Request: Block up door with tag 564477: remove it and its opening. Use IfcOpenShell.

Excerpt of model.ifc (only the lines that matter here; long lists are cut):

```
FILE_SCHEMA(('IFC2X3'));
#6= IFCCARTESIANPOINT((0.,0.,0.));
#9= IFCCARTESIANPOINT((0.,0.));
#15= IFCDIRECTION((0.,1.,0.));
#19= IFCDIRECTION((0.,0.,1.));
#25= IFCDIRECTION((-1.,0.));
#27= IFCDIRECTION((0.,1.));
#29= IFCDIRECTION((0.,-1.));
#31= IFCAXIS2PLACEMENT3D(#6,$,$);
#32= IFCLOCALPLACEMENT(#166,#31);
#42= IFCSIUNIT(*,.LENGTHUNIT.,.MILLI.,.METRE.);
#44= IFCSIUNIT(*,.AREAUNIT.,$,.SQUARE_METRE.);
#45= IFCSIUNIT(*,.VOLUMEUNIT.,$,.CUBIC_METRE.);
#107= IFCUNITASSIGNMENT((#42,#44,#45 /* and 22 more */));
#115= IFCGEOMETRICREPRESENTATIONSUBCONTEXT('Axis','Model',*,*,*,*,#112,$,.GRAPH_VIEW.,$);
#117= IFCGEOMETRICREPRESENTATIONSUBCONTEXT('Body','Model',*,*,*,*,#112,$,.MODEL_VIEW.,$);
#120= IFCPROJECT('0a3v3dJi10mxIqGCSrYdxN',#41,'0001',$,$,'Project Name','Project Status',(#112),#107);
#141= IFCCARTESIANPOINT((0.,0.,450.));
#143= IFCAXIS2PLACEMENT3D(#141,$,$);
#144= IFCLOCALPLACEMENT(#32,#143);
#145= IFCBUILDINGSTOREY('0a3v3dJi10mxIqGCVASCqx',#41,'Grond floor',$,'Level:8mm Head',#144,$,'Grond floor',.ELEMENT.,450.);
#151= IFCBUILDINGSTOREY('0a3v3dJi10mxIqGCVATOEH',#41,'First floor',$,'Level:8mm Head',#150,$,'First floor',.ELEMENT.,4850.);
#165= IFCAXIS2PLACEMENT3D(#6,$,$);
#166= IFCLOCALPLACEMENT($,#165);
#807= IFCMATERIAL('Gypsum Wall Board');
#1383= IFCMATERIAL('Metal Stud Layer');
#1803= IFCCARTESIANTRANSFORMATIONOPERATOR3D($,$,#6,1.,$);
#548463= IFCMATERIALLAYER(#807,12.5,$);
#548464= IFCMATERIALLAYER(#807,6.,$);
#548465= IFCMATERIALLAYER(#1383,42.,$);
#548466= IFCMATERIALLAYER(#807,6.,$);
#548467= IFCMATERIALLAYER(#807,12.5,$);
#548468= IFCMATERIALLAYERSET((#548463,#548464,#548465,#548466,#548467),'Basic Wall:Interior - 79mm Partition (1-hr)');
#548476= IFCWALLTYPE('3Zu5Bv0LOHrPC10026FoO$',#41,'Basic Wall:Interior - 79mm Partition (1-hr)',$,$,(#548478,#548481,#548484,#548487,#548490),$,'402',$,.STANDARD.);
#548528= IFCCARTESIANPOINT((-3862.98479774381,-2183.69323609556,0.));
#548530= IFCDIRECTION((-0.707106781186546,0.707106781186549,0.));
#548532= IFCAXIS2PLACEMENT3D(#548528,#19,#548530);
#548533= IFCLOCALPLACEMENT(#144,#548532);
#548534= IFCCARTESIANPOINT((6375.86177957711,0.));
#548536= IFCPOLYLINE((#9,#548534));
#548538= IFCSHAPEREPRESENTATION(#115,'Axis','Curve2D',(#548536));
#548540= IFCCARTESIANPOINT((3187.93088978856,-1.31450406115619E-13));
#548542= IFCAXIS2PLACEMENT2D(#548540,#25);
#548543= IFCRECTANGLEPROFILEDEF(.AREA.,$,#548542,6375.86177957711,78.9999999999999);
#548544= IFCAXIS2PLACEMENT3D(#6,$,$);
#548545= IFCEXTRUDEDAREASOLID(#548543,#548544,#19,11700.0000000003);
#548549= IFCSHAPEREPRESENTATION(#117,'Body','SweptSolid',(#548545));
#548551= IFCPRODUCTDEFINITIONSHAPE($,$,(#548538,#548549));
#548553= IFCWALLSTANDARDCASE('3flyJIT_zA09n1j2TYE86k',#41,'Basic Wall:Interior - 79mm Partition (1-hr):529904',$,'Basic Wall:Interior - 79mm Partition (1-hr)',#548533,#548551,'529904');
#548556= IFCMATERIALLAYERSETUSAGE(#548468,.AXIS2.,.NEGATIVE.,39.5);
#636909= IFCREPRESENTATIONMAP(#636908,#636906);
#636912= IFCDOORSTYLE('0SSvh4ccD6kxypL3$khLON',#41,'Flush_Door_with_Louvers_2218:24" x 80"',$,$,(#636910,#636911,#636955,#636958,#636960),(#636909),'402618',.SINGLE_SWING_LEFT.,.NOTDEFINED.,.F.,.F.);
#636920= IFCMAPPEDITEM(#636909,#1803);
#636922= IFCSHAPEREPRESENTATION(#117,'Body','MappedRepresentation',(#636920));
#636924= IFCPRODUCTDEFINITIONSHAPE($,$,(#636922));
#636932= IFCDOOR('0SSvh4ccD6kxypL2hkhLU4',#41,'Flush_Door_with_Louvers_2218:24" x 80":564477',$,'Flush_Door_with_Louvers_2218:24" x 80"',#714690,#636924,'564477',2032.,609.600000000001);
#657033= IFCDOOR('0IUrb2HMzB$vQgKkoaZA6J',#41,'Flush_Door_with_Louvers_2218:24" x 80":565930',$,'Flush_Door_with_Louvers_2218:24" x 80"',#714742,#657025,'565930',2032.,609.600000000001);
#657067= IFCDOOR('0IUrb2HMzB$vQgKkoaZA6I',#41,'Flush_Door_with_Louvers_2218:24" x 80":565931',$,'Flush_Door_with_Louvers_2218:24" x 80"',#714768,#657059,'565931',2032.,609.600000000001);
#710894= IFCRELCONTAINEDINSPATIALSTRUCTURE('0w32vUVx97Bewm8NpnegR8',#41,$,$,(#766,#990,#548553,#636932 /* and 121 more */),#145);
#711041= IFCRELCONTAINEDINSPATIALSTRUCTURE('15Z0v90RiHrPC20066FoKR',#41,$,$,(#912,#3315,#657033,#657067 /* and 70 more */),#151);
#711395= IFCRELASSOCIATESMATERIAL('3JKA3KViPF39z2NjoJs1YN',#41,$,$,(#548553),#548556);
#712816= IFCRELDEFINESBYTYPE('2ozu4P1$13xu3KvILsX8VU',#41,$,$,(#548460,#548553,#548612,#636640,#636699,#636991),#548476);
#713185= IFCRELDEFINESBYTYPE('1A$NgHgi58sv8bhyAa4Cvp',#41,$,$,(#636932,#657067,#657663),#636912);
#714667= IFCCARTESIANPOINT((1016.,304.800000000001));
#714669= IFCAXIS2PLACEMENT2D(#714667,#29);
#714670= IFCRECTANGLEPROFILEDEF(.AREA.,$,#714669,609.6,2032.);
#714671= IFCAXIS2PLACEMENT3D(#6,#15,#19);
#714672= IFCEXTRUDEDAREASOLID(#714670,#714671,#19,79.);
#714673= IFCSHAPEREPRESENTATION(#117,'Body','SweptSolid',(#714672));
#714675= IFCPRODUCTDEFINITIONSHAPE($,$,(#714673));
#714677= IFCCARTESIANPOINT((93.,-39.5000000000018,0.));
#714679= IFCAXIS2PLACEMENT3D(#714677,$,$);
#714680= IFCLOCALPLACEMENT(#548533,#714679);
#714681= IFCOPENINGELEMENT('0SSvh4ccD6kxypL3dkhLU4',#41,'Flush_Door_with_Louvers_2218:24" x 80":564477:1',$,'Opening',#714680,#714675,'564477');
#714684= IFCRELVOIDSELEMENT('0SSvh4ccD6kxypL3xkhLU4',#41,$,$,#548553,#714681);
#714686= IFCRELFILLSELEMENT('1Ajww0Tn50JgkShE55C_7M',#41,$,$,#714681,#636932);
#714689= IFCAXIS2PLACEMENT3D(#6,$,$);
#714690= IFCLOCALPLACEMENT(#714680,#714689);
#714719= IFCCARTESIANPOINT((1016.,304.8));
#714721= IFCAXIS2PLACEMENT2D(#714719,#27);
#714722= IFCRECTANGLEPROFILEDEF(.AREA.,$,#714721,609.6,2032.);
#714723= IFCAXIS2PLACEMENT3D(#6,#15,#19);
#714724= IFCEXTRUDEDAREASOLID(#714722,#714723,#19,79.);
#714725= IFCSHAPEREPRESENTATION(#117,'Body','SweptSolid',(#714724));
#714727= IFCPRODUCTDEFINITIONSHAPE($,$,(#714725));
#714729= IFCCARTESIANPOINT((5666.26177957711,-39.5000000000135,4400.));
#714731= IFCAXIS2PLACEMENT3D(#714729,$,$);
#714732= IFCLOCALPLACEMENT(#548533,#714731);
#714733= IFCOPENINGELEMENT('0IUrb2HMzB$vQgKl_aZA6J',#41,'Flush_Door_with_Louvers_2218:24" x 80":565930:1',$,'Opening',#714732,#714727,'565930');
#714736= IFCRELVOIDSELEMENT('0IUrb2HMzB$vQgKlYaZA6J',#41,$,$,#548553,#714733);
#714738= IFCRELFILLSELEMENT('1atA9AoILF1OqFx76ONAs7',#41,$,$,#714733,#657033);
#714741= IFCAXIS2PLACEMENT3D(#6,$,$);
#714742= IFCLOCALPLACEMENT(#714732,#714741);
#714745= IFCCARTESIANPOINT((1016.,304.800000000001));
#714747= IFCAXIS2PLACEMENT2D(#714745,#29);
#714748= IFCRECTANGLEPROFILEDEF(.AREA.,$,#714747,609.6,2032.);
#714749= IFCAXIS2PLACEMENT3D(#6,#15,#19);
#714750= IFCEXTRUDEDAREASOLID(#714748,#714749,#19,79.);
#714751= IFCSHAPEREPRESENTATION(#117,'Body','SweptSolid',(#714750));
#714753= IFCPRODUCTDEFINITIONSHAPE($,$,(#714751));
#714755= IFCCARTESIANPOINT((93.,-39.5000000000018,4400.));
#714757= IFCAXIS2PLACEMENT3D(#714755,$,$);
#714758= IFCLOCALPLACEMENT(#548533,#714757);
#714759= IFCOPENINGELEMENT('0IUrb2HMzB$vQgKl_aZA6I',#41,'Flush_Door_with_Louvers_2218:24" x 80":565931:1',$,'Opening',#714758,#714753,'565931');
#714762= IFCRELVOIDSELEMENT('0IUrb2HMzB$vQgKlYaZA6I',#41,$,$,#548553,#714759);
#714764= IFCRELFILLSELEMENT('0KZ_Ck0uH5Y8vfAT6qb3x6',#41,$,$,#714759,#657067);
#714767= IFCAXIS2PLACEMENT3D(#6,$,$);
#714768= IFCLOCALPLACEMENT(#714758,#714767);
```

```python
import ifcopenshell
import ifcopenshell.api.feature
import ifcopenshell.api.root
import ifcopenshell.geom
import ifcopenshell.util.shape

model = ifcopenshell.open("model.ifc")
settings = ifcopenshell.geom.settings()


def volume(element):
    """Net volume in cubic metres, openings subtracted."""
    shape = ifcopenshell.geom.create_shape(settings, element)
    return ifcopenshell.util.shape.get_volume(shape.geometry)


door = model.by_guid("0SSvh4ccD6kxypL2hkhLU4")
opening = door.FillsVoids[0].RelatingOpeningElement
wall = opening.VoidsElements[0].RelatingBuildingElement
before = volume(wall)

ifcopenshell.api.root.remove_product(model, product=door)
ifcopenshell.api.feature.remove_feature(model, feature=opening)

after = volume(wall)

print(f"wall volume {before:.3f} -> {after:.3f} m3")

model.write("model-out.ifc")
```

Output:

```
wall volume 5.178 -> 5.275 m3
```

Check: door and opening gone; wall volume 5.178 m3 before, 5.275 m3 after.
